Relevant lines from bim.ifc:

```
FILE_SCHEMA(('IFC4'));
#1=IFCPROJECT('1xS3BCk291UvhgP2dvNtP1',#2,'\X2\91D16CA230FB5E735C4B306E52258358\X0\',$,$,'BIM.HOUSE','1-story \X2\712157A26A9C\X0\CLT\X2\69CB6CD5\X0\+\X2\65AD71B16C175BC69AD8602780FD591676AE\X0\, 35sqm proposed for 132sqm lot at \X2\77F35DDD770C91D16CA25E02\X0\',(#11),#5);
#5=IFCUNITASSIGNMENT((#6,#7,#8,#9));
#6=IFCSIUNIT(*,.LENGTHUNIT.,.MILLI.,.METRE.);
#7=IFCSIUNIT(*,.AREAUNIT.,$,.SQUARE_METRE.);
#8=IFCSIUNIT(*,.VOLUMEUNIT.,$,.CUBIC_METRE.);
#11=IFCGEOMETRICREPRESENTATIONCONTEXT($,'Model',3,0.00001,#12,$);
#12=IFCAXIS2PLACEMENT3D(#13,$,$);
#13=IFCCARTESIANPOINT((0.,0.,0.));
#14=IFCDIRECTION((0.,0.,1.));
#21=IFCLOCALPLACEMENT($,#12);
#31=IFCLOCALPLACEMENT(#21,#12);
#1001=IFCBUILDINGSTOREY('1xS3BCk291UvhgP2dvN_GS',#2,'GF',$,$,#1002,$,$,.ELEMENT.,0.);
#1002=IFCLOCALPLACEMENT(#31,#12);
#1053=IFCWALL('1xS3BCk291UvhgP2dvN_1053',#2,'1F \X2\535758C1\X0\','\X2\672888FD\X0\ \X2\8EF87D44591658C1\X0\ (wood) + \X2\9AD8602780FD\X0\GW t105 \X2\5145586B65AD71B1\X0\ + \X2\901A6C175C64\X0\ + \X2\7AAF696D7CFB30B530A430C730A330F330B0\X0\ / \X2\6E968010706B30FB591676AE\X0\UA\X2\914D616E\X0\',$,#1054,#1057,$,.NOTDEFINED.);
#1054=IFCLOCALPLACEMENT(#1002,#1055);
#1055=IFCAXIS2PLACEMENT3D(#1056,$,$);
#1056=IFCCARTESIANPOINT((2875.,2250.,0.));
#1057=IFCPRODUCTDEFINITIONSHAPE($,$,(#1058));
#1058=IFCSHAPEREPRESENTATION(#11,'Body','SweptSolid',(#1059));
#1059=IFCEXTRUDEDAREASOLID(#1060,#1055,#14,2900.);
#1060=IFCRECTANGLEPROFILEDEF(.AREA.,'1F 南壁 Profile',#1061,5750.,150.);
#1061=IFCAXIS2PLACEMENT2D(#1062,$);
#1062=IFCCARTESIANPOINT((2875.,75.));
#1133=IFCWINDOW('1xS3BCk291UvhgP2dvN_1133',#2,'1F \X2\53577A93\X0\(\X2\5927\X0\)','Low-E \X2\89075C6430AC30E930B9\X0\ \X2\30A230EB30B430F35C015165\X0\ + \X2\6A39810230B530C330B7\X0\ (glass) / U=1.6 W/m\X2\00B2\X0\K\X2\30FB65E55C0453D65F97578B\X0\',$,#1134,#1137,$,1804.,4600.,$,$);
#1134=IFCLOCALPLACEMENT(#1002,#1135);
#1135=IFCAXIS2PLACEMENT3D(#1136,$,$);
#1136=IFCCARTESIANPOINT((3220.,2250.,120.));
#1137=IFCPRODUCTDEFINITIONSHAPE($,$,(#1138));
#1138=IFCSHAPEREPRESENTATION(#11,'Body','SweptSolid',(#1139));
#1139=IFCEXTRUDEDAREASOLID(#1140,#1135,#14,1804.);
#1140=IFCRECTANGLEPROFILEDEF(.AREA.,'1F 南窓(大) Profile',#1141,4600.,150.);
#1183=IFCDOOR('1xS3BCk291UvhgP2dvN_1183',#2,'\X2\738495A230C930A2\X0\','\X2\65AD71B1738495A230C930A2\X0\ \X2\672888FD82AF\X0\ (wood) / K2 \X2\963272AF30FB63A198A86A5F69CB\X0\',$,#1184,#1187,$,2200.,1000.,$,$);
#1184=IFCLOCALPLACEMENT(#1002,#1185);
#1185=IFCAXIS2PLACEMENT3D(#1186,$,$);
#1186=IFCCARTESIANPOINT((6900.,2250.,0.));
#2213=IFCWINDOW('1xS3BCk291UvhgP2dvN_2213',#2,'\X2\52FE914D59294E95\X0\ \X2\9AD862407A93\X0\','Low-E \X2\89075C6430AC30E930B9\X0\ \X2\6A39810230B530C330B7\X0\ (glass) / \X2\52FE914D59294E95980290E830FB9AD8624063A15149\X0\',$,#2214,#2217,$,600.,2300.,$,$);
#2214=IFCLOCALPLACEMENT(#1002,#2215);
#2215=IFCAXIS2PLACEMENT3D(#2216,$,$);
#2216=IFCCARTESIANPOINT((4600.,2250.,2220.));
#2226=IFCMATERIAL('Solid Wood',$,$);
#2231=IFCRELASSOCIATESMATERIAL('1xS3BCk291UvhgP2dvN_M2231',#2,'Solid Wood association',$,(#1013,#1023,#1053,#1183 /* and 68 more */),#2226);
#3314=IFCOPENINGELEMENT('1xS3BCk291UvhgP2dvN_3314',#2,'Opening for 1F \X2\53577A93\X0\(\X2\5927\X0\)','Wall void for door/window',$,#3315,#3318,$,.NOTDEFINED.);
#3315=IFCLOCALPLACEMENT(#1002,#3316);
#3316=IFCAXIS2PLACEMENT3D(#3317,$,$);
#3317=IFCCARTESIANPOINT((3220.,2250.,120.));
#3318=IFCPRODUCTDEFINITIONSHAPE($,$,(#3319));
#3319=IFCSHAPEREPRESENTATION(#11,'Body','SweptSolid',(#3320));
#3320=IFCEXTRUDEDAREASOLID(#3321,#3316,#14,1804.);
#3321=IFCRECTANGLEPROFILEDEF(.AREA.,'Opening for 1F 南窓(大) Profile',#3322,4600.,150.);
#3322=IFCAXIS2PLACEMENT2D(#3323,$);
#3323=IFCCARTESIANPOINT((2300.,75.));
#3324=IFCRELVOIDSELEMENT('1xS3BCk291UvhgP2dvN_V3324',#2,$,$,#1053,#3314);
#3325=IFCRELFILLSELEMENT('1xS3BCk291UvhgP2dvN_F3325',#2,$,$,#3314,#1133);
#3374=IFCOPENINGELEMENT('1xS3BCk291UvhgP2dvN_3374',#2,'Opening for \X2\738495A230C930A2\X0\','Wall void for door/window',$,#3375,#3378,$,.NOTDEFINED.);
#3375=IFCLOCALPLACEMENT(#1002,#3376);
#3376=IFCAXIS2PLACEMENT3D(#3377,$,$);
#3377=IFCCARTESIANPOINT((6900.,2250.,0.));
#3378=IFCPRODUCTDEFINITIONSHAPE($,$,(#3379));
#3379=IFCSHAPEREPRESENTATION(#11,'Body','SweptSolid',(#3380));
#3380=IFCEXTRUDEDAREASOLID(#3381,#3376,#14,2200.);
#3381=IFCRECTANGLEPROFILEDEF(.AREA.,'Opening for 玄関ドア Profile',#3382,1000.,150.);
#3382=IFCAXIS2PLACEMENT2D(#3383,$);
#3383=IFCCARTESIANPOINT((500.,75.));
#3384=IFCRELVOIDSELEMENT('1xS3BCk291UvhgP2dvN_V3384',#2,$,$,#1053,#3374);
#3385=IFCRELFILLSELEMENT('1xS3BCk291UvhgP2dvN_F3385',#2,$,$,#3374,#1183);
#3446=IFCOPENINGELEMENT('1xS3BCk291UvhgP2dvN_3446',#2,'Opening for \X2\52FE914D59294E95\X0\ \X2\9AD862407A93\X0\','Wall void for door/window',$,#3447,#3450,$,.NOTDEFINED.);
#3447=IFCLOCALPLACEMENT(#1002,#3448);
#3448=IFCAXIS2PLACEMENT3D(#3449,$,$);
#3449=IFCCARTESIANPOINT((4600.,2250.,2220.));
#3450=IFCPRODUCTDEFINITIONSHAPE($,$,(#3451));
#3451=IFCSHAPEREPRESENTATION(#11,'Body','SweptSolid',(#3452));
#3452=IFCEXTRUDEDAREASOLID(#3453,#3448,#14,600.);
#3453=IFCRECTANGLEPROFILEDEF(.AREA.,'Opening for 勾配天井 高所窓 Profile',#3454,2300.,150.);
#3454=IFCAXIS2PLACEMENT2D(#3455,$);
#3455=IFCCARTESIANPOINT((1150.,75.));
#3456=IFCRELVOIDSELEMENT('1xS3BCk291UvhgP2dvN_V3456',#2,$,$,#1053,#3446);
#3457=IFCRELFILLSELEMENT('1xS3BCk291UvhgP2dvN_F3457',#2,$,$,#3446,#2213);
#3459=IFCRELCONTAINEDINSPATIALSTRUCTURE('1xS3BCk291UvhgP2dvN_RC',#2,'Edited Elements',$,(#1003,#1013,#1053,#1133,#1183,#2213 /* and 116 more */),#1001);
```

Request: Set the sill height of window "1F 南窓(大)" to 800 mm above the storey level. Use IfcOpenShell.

```python
import numpy as np
import ifcopenshell
import ifcopenshell.api.geometry
import ifcopenshell.geom
import ifcopenshell.util.element
import ifcopenshell.util.placement
import ifcopenshell.util.shape
import ifcopenshell.util.unit

model = ifcopenshell.open("bim.ifc")
unit_scale = ifcopenshell.util.unit.calculate_unit_scale(model)

window = model.by_guid("1xS3BCk291UvhgP2dvN_1133")
opening = window.FillsVoids[0].RelatingOpeningElement
storey = ifcopenshell.util.element.get_container(window, ifc_class="IfcBuildingStorey")
level = ifcopenshell.util.placement.get_local_placement(storey.ObjectPlacement)[2, 3]

# The opening's origin need not be at the sill, so measure its lowest point.
shape = ifcopenshell.geom.create_shape(ifcopenshell.geom.settings(), opening)
bottom = ifcopenshell.util.shape.get_shape_bottom_elevation(shape, shape.geometry) / unit_scale
dz = level + 800.0 - bottom

shift = np.array([0.0, 0.0, dz])
# The window is not placed relative to its opening, so move both.
for product in (opening, window):
    matrix = ifcopenshell.util.placement.get_local_placement(product.ObjectPlacement)
    matrix[:3, 3] += shift
    ifcopenshell.api.geometry.edit_object_placement(model, product=product, matrix=matrix, is_si=False)

print(f"moved by {dz * unit_scale:+.3f} m")

model.write("bim_v2.ifc")
```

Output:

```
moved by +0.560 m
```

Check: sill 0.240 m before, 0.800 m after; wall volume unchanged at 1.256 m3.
